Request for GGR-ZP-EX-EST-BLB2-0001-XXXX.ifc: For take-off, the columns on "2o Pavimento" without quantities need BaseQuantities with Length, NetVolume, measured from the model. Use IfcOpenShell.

First a look at what the model holds.

```python
import ifcopenshell
import ifcopenshell.util.element
import ifcopenshell.util.unit

model = ifcopenshell.open("GGR-ZP-EX-EST-BLB2-0001-XXXX.ifc")
print(model.schema)
for unit_type in ("LENGTHUNIT", "AREAUNIT", "VOLUMEUNIT"):
    print(unit_type, ifcopenshell.util.unit.calculate_unit_scale(model, unit_type))
storey = next(s for s in model.by_type("IfcBuildingStorey") if s.Name == "2o Pavimento")
columns = [e for e in ifcopenshell.util.element.get_decomposition(storey) if e.is_a("IfcColumn")]
for e in sorted(columns, key=lambda e: e.id()):
    print(e.id(), e.is_a(), e.Name, list(ifcopenshell.util.element.get_psets(e, qtos_only=True)), sep=" | ")
```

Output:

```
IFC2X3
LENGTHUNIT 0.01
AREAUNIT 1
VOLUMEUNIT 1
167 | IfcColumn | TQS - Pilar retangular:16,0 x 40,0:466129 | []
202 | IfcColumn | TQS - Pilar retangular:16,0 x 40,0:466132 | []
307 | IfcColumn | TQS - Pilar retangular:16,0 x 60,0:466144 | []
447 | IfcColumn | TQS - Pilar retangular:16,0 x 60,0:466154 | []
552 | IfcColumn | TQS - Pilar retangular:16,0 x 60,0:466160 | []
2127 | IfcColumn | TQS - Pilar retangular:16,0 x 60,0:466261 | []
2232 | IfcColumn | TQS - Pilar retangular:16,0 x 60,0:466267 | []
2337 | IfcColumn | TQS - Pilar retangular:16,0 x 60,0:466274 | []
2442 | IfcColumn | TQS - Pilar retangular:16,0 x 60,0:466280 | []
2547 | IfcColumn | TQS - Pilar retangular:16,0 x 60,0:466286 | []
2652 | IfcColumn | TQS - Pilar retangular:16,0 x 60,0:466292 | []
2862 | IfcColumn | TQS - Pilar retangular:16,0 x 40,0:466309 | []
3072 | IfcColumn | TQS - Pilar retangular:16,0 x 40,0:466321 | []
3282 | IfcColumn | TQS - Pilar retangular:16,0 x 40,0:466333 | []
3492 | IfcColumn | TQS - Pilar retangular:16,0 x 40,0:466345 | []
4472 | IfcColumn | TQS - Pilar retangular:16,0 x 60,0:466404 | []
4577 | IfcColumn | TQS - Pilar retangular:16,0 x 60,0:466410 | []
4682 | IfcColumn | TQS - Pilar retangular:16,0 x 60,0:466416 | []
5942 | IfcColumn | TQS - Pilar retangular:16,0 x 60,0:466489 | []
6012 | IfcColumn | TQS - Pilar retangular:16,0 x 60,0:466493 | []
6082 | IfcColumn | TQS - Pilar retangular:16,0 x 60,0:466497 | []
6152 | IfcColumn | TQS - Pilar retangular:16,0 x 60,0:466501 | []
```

```python
import ifcopenshell
import ifcopenshell.api.pset
import ifcopenshell.geom
import ifcopenshell.util.element
import ifcopenshell.util.shape
import ifcopenshell.util.unit

model = ifcopenshell.open("GGR-ZP-EX-EST-BLB2-0001-XXXX.ifc")
unit_scale = ifcopenshell.util.unit.calculate_unit_scale(model)
volume_scale = ifcopenshell.util.unit.calculate_unit_scale(model, "VOLUMEUNIT")
settings = ifcopenshell.geom.settings()

storey = next(s for s in model.by_type("IfcBuildingStorey") if s.Name == "2o Pavimento")
columns = [e for e in ifcopenshell.util.element.get_decomposition(storey) if e.is_a("IfcColumn")]

for e in sorted(columns, key=lambda e: e.id()):
    if ifcopenshell.util.element.get_psets(e, qtos_only=True, should_inherit=False):
        continue
    # Geometry comes back in metres, in the element's own axes.
    shape = ifcopenshell.geom.create_shape(settings, e)
    values = {
        "Length": ifcopenshell.util.shape.get_z(shape.geometry) / unit_scale,
        "NetVolume": ifcopenshell.util.shape.get_volume(shape.geometry) / volume_scale,
    }
    qto = ifcopenshell.api.pset.add_qto(model, product=e, name="BaseQuantities")
    ifcopenshell.api.pset.edit_qto(model, qto=qto, properties=values)
    print(e.id(), {k: round(v, 3) for k, v in values.items()})

model.write("GGR-ZP-EX-EST-BLB2-0001-XXXX_rev.ifc")
```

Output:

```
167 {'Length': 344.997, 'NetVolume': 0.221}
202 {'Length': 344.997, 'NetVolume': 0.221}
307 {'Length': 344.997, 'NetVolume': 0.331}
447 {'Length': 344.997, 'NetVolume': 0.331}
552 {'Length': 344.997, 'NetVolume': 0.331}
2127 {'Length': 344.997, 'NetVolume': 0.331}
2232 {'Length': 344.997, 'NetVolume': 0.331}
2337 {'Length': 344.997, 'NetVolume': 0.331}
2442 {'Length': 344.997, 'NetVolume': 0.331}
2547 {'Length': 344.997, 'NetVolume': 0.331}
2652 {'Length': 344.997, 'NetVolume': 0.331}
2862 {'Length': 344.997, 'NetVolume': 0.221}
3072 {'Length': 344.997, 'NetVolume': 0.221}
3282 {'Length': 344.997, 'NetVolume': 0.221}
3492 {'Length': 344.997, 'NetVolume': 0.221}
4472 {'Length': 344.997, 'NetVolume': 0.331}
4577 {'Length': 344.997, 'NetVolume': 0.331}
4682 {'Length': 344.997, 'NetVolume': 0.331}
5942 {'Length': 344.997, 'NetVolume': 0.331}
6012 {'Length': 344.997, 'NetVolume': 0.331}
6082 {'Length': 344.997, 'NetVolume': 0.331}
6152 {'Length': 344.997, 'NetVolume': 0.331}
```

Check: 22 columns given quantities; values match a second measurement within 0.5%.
